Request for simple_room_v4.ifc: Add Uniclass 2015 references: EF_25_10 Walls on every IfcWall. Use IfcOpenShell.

First a look at what the model holds.

```python
import ifcopenshell

model = ifcopenshell.open("simple_room_v4.ifc")
print(model.schema)
print("classifications:", [c.Name for c in model.by_type("IfcClassification")])
for ifc_class in ("IfcDoor", "IfcRoof", "IfcStair", "IfcWall", "IfcWindow"):
    print(ifc_class, len(model.by_type(ifc_class)))
```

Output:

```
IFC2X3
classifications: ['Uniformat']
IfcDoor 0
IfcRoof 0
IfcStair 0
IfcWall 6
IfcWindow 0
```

```python
import ifcopenshell
import ifcopenshell.api.classification

model = ifcopenshell.open("simple_room_v4.ifc")

# IFC2X3 requires Source and Edition and has no link from the project to the system.
system = model.create_entity("IfcClassification", Source="NBS", Edition="2015", Name="Uniclass 2015")

codes = {
    "IfcWall": ("EF_25_10", "Walls"),
}
for ifc_class, (code, name) in codes.items():
    products = model.by_type(ifc_class)
    ifcopenshell.api.classification.add_reference(
        model, products=products, classification=system, identification=code, name=name
    )
    print(code, len(products))

model.write("simple_room_v4_v2.ifc")
```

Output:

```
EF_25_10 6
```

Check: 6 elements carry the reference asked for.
